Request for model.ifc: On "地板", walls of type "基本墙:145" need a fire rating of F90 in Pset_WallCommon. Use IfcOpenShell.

First a look at what the model holds.

```python
import ifcopenshell
import ifcopenshell.util.element

model = ifcopenshell.open("model.ifc")
print(model.schema)
storey = next(s for s in model.by_type("IfcBuildingStorey") if s.Name == "地板")
walls = [e for e in ifcopenshell.util.element.get_decomposition(storey) if e.is_a("IfcWall")]
seen = {}
for e in walls:
    element_type = ifcopenshell.util.element.get_type(e)
    key = (element_type.Name if element_type != e and element_type else None, ifcopenshell.util.element.get_pset(e, "Pset_WallCommon", "FireRating"))
    seen[key] = seen.get(key, 0) + 1
for (name, value), count in sorted(seen.items(), key=str):
    print(count, "x", name, "|", value)
```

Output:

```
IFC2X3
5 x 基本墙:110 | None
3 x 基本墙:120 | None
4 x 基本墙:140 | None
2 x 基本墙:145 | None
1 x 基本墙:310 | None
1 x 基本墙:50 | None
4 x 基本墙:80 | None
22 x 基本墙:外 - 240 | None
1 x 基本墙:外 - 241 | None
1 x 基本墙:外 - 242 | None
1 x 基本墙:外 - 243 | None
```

```python
import ifcopenshell
import ifcopenshell.api.pset
import ifcopenshell.util.element

model = ifcopenshell.open("model.ifc")

storey = next(s for s in model.by_type("IfcBuildingStorey") if s.Name == "地板")
walls = [e for e in ifcopenshell.util.element.get_decomposition(storey) if e.is_a("IfcWall")]

count = 0
for e in walls:
    element_type = ifcopenshell.util.element.get_type(e)
    if element_type in (None, e) or element_type.Name != "基本墙:145":
        continue
    # add_pset returns the element's existing set when there is one.
    pset = ifcopenshell.api.pset.add_pset(model, product=e, name="Pset_WallCommon")
    ifcopenshell.api.pset.edit_pset(model, pset=pset, properties={"FireRating": "F90"})
    count += 1

print(count, "walls updated")

model.write("model_updated.ifc")
```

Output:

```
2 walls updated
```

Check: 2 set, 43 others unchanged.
